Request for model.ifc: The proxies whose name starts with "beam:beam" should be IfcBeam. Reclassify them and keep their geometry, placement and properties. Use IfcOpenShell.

First a look at what the model holds.

```python
import re

import ifcopenshell

model = ifcopenshell.open("model.ifc")
print(model.schema)
seen = {}
for e in model.by_type("IfcBuildingElementProxy"):
    name = re.sub(r":\d+(:\d+)?$", "", e.Name or "")  # drop the element id that some exporters append
    seen[name] = seen.get(name, 0) + 1
for name, count in sorted(seen.items()):
    print(count, "x", name)
```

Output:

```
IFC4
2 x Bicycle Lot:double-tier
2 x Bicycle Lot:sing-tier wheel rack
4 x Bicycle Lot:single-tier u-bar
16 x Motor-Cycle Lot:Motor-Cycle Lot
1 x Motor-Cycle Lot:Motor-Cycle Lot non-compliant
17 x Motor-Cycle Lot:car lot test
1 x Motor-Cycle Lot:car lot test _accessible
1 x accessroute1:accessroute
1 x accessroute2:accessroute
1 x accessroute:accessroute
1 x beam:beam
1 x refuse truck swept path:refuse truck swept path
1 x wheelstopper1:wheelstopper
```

```python
import ifcopenshell
import ifcopenshell.api.root

model = ifcopenshell.open("model.ifc")

proxies = [e.id() for e in model.by_type("IfcBuildingElementProxy") if (e.Name or "").startswith("beam:beam")]
for step_id in proxies:
    proxy = model.by_id(step_id)
    # Reclassifying a typed element also reclassifies its type and the type's other occurrences.
    if proxy.is_a("IfcBuildingElementProxy"):
        ifcopenshell.api.root.reassign_class(model, product=proxy, ifc_class="IfcBeam")

print(sum(model.by_id(i).is_a("IfcBeam") for i in proxies), "reclassified")

model.write("model_updated.ifc")
```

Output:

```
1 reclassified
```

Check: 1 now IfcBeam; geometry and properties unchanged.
